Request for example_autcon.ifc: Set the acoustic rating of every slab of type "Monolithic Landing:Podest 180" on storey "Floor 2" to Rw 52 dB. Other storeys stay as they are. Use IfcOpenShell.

First a look at what the model holds.

```python
import ifcopenshell
import ifcopenshell.util.element

model = ifcopenshell.open("example_autcon.ifc")
print(model.schema)
storey = next(s for s in model.by_type("IfcBuildingStorey") if s.Name == "Floor 2")
slabs = [e for e in ifcopenshell.util.element.get_decomposition(storey) if e.is_a("IfcSlab")]
seen = {}
for e in slabs:
    element_type = ifcopenshell.util.element.get_type(e)
    key = (element_type.Name if element_type != e and element_type else None, ifcopenshell.util.element.get_pset(e, "Pset_SlabCommon", "AcousticRating"))
    seen[key] = seen.get(key, 0) + 1
for (name, value), count in sorted(seen.items(), key=str):
    print(count, "x", name, "|", value)
```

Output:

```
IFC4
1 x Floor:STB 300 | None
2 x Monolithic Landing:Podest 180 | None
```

```python
import ifcopenshell
import ifcopenshell.api.pset
import ifcopenshell.util.element

model = ifcopenshell.open("example_autcon.ifc")

storey = next(s for s in model.by_type("IfcBuildingStorey") if s.Name == "Floor 2")
slabs = [e for e in ifcopenshell.util.element.get_decomposition(storey) if e.is_a("IfcSlab")]

count = 0
for e in slabs:
    element_type = ifcopenshell.util.element.get_type(e)
    if element_type in (None, e) or element_type.Name != "Monolithic Landing:Podest 180":
        continue
    # add_pset returns the element's existing set when there is one.
    pset = ifcopenshell.api.pset.add_pset(model, product=e, name="Pset_SlabCommon")
    ifcopenshell.api.pset.edit_pset(model, pset=pset, properties={"AcousticRating": "Rw 52 dB"})
    count += 1

print(count, "slabs updated")

model.write("example_autcon_edited.ifc")
```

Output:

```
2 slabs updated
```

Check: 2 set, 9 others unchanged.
